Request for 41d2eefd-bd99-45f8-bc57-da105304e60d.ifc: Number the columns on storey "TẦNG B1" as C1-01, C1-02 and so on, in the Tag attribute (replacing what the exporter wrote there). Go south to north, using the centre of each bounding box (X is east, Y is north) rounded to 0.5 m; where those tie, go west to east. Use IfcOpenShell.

First a look at what the model holds.

```python
import ifcopenshell
import ifcopenshell.util.element
import ifcopenshell.util.placement

model = ifcopenshell.open("41d2eefd-bd99-45f8-bc57-da105304e60d.ifc")
print(model.schema)
storey = next(s for s in model.by_type("IfcBuildingStorey") if s.Name == "TẦNG B1")
columns = [e for e in ifcopenshell.util.element.get_decomposition(storey) if e.is_a("IfcColumn")]
for e in sorted(columns, key=lambda e: e.id()):
    origin = ifcopenshell.util.placement.get_local_placement(e.ObjectPlacement)[:3, 3]
    print(e.id(), e.Tag, e.Name, origin.round(2) + 0.0, sep=" | ")
```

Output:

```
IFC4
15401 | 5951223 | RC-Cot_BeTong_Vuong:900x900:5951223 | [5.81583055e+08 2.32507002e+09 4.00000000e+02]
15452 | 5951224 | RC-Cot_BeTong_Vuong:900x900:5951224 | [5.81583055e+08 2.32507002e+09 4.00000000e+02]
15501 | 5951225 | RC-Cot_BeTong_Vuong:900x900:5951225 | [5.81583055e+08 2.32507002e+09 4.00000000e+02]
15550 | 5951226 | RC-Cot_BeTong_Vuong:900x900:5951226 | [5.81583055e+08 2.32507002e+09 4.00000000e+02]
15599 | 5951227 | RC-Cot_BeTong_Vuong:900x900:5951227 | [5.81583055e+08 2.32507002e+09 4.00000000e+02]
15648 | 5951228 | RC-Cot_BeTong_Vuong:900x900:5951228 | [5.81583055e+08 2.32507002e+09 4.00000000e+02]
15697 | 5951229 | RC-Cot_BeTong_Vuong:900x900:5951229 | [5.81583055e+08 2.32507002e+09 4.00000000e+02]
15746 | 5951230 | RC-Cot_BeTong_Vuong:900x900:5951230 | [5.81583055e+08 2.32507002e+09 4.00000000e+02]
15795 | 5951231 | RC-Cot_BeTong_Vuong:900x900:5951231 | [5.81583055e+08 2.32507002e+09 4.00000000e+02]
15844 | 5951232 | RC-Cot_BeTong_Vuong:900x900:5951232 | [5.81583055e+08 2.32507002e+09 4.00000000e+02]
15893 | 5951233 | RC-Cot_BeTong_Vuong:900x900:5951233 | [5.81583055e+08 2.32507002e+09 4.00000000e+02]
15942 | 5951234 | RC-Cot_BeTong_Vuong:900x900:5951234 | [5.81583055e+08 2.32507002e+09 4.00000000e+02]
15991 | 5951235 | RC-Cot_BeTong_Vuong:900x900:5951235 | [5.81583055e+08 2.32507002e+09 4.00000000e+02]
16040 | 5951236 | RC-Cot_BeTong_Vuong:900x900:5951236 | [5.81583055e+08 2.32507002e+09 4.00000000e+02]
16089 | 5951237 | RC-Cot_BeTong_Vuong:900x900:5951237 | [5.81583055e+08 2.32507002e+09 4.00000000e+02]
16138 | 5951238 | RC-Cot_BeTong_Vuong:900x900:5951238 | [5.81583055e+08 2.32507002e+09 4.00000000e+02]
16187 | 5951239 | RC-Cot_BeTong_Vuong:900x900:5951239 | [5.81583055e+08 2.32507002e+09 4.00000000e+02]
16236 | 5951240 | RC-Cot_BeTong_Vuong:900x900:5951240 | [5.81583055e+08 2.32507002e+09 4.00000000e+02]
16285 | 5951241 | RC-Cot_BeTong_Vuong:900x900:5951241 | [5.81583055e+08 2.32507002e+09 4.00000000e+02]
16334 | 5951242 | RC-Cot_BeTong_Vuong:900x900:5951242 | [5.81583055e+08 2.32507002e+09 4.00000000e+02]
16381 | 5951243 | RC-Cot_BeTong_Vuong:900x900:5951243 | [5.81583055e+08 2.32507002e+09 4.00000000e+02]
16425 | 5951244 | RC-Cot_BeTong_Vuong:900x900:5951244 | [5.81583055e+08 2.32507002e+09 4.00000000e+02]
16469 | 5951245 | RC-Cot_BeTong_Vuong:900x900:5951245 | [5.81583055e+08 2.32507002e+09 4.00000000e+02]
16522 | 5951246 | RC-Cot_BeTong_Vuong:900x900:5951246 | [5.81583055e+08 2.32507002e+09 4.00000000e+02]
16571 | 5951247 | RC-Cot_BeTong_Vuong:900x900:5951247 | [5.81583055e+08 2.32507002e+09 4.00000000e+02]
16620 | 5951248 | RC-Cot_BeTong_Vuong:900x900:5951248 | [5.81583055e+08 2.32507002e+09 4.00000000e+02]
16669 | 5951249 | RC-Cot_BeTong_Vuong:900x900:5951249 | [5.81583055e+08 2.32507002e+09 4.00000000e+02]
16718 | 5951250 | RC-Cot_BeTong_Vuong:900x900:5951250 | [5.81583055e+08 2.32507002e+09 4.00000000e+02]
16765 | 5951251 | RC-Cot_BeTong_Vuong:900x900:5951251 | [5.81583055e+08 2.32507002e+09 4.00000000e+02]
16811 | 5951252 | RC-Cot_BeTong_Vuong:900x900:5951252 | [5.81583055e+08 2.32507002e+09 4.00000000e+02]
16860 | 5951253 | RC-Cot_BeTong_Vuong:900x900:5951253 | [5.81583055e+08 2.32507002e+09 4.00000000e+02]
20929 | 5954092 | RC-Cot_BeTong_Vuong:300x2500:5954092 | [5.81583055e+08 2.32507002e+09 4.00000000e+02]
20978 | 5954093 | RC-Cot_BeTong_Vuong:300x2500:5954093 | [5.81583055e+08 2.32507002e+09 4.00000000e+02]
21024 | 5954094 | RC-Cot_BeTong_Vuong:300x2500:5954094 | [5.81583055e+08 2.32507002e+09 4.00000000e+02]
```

```python
import ifcopenshell
import ifcopenshell.geom
import ifcopenshell.util.element
import ifcopenshell.util.shape

model = ifcopenshell.open("41d2eefd-bd99-45f8-bc57-da105304e60d.ifc")
settings = ifcopenshell.geom.settings()
settings.set("use-world-coords", True)


def centre(element):
    shape = ifcopenshell.geom.create_shape(settings, element)
    return ifcopenshell.util.shape.get_bbox_centroid(shape.geometry)


storey = next(s for s in model.by_type("IfcBuildingStorey") if s.Name == "TẦNG B1")
columns = [e for e in ifcopenshell.util.element.get_decomposition(storey) if e.is_a("IfcColumn")]

# Insertion points can sit at a corner or the storey origin, so sort by the geometry (in metres).
centres = {e: centre(e) for e in columns}
columns.sort(key=lambda e: (round(centres[e][1] / 0.5), centres[e][0]))

for i, e in enumerate(columns, start=1):
    number = f"C1-{i:02d}"
    e.Tag = number
    print(e.id(), number)

model.write("41d2eefd-bd99-45f8-bc57-da105304e60d_updated.ifc")
```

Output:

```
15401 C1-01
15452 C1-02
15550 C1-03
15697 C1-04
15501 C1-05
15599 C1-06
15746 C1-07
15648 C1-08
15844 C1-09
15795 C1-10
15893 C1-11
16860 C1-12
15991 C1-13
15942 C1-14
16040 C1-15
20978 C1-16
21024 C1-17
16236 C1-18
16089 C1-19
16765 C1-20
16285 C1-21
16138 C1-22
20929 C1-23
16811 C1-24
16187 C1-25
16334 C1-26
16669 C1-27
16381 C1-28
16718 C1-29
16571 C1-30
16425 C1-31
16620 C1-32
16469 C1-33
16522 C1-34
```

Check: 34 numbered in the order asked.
